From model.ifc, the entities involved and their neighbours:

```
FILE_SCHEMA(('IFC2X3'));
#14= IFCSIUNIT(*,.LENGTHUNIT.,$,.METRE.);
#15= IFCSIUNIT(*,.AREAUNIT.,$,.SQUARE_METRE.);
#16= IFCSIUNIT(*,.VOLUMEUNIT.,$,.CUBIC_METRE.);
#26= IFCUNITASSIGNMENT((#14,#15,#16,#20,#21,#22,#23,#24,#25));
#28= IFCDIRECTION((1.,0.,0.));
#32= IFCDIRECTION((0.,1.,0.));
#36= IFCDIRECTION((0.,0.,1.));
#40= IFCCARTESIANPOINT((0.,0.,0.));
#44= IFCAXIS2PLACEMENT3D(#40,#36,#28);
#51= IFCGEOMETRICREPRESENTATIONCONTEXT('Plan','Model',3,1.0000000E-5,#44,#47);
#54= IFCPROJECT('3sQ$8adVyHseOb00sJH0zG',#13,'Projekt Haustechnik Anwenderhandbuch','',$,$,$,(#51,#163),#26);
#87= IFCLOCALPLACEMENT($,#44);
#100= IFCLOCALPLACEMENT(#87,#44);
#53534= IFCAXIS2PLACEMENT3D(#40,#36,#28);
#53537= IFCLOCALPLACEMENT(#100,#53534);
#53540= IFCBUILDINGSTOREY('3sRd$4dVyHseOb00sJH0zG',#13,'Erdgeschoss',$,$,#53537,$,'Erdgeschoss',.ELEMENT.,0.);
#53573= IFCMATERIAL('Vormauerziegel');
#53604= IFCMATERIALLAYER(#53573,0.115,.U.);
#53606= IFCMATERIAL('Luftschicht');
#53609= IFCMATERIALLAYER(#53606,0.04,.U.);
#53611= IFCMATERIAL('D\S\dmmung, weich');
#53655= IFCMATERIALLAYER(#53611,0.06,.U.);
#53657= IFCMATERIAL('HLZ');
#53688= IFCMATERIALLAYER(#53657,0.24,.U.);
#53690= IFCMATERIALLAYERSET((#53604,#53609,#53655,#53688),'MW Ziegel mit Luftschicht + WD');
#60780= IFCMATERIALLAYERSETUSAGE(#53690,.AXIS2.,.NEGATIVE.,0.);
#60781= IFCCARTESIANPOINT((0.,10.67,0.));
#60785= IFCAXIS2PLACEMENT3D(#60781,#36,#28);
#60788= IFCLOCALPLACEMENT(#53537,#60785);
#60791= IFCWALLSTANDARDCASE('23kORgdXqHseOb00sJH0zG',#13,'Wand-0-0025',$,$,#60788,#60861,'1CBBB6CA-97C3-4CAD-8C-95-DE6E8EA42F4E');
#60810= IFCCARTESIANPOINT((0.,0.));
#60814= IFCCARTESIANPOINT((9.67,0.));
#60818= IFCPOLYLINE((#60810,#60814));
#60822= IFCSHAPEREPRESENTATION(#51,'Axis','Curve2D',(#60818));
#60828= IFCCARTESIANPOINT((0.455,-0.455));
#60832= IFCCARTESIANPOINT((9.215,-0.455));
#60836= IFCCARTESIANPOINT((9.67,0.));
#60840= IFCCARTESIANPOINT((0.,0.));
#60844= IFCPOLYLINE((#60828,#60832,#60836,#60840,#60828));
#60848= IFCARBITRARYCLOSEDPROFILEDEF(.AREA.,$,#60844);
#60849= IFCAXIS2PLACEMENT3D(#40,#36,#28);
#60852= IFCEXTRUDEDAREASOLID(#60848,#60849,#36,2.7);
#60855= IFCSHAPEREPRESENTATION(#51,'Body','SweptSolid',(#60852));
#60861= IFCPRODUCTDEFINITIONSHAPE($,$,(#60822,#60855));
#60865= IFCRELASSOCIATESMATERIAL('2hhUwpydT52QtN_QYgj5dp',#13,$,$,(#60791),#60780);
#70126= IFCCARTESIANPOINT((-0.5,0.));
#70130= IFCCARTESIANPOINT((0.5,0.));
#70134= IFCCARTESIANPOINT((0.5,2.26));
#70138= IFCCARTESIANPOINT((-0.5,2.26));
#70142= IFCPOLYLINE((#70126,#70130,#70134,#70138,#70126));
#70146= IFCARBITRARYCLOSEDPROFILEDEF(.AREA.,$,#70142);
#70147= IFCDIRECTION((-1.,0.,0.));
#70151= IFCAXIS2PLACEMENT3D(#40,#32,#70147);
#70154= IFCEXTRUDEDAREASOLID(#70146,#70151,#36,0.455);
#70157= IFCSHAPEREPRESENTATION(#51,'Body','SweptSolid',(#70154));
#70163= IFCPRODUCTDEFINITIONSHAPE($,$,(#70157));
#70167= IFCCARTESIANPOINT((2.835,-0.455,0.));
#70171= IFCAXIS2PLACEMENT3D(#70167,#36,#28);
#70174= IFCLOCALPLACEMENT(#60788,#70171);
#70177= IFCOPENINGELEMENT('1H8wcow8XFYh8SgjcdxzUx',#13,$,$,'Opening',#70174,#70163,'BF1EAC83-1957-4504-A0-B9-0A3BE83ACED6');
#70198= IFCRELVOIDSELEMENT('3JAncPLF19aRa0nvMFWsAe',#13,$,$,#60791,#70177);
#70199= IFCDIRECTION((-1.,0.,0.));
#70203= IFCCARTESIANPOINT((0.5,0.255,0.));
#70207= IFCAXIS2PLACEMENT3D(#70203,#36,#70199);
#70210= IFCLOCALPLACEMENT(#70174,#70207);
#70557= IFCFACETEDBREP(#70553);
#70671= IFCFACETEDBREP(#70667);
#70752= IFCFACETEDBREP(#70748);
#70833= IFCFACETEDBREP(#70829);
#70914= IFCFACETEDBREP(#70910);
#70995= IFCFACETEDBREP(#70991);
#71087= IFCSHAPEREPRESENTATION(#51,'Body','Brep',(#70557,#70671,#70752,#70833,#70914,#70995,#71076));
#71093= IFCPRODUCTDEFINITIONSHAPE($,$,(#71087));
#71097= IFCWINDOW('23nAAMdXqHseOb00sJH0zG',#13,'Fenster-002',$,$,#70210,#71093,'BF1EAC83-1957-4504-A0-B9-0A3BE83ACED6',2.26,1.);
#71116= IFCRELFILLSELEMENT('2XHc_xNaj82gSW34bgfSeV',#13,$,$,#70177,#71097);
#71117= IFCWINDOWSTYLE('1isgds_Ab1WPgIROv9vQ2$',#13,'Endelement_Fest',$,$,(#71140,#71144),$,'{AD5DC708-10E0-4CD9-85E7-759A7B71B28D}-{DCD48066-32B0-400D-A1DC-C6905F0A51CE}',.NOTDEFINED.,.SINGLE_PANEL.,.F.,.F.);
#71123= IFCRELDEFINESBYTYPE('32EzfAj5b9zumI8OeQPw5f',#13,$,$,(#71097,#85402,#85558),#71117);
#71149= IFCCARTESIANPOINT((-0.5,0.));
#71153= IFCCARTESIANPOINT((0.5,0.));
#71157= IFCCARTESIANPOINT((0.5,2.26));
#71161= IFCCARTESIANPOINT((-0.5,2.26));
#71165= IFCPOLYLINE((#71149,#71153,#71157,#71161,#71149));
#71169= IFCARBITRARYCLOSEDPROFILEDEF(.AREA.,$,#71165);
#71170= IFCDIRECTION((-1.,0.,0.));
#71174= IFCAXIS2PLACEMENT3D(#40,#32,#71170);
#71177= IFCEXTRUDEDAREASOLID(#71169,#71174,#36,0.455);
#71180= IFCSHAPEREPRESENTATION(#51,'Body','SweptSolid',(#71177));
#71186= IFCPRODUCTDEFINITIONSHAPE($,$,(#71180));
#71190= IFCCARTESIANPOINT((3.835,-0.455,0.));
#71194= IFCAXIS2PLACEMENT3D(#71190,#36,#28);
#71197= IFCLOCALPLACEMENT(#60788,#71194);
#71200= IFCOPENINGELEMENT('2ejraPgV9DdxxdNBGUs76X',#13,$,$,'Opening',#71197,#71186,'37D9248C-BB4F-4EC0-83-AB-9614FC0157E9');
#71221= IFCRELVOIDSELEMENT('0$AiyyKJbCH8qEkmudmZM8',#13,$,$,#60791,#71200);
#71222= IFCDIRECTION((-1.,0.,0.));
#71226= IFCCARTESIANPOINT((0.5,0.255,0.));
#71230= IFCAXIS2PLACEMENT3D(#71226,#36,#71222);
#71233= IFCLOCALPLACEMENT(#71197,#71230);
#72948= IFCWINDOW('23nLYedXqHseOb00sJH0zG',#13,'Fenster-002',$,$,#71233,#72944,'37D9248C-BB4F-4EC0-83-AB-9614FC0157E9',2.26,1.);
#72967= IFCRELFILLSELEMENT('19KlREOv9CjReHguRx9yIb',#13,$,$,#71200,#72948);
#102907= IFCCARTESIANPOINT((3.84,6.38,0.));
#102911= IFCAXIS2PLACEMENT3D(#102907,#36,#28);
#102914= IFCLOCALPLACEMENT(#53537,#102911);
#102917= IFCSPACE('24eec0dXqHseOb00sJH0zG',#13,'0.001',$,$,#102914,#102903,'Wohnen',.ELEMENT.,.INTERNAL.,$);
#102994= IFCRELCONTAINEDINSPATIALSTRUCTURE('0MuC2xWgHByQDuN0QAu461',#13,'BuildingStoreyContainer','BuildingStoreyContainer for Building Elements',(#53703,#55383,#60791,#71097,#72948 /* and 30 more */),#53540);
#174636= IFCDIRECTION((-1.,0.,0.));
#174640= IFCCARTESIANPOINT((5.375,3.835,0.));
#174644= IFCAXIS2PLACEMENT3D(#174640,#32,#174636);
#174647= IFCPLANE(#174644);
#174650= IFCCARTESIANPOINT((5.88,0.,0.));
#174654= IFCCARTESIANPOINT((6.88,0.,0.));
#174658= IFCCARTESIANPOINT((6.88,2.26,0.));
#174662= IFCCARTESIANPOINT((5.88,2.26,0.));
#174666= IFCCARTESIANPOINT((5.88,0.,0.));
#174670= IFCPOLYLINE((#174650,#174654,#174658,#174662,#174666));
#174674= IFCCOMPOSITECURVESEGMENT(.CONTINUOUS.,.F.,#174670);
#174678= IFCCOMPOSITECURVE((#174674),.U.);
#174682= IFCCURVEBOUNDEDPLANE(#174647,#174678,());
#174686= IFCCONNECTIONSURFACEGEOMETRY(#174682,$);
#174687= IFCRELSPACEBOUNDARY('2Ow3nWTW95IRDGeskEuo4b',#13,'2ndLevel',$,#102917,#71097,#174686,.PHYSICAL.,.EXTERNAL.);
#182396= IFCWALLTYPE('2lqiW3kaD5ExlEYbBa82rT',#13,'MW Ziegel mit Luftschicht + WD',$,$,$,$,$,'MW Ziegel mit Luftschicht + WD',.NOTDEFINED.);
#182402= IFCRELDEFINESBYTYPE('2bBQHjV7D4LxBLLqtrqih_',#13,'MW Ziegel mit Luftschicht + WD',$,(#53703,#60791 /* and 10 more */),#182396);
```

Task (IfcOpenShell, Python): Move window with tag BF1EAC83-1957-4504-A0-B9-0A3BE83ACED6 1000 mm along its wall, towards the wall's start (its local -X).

```python
import numpy as np
import ifcopenshell
import ifcopenshell.api.geometry
import ifcopenshell.util.placement
import ifcopenshell.util.unit

model = ifcopenshell.open("model.ifc")
unit_scale = ifcopenshell.util.unit.calculate_unit_scale(model)

window = model.by_guid("23nAAMdXqHseOb00sJH0zG")
opening = window.FillsVoids[0].RelatingOpeningElement
wall = opening.VoidsElements[0].RelatingBuildingElement

wall_matrix = ifcopenshell.util.placement.get_local_placement(wall.ObjectPlacement)
shift = wall_matrix[:3, 0] * -1 / unit_scale
before = ifcopenshell.util.placement.get_local_placement(window.ObjectPlacement)[:3, 3].copy()

# The window is placed relative to its opening, so it follows when the opening moves.
matrix = ifcopenshell.util.placement.get_local_placement(opening.ObjectPlacement)
matrix[:3, 3] += shift
ifcopenshell.api.geometry.edit_object_placement(
    model, product=opening, matrix=matrix, is_si=False, should_transform_children=True
)

# Space boundary surfaces are stored in each space's coordinates; move them too.
for rel in window.ProvidesBoundaries:
    if not rel.ConnectionGeometry:
        continue
    surface = rel.ConnectionGeometry.SurfaceOnRelatingElement.BasisSurface
    space_matrix = ifcopenshell.util.placement.get_local_placement(rel.RelatingSpace.ObjectPlacement)
    point = np.array(surface.Position.Location.Coordinates) + space_matrix[:3, :3].T @ shift
    surface.Position = model.createIfcAxis2Placement3D(
        model.createIfcCartesianPoint(point.tolist()), surface.Position.Axis, surface.Position.RefDirection
    )

after = ifcopenshell.util.placement.get_local_placement(window.ObjectPlacement)[:3, 3]
print("window moved by", (after - before).round(3) + 0.0)

model.write("model_updated.ifc")
```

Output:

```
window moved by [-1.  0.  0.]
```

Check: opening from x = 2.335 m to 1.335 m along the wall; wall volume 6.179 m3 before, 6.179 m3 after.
